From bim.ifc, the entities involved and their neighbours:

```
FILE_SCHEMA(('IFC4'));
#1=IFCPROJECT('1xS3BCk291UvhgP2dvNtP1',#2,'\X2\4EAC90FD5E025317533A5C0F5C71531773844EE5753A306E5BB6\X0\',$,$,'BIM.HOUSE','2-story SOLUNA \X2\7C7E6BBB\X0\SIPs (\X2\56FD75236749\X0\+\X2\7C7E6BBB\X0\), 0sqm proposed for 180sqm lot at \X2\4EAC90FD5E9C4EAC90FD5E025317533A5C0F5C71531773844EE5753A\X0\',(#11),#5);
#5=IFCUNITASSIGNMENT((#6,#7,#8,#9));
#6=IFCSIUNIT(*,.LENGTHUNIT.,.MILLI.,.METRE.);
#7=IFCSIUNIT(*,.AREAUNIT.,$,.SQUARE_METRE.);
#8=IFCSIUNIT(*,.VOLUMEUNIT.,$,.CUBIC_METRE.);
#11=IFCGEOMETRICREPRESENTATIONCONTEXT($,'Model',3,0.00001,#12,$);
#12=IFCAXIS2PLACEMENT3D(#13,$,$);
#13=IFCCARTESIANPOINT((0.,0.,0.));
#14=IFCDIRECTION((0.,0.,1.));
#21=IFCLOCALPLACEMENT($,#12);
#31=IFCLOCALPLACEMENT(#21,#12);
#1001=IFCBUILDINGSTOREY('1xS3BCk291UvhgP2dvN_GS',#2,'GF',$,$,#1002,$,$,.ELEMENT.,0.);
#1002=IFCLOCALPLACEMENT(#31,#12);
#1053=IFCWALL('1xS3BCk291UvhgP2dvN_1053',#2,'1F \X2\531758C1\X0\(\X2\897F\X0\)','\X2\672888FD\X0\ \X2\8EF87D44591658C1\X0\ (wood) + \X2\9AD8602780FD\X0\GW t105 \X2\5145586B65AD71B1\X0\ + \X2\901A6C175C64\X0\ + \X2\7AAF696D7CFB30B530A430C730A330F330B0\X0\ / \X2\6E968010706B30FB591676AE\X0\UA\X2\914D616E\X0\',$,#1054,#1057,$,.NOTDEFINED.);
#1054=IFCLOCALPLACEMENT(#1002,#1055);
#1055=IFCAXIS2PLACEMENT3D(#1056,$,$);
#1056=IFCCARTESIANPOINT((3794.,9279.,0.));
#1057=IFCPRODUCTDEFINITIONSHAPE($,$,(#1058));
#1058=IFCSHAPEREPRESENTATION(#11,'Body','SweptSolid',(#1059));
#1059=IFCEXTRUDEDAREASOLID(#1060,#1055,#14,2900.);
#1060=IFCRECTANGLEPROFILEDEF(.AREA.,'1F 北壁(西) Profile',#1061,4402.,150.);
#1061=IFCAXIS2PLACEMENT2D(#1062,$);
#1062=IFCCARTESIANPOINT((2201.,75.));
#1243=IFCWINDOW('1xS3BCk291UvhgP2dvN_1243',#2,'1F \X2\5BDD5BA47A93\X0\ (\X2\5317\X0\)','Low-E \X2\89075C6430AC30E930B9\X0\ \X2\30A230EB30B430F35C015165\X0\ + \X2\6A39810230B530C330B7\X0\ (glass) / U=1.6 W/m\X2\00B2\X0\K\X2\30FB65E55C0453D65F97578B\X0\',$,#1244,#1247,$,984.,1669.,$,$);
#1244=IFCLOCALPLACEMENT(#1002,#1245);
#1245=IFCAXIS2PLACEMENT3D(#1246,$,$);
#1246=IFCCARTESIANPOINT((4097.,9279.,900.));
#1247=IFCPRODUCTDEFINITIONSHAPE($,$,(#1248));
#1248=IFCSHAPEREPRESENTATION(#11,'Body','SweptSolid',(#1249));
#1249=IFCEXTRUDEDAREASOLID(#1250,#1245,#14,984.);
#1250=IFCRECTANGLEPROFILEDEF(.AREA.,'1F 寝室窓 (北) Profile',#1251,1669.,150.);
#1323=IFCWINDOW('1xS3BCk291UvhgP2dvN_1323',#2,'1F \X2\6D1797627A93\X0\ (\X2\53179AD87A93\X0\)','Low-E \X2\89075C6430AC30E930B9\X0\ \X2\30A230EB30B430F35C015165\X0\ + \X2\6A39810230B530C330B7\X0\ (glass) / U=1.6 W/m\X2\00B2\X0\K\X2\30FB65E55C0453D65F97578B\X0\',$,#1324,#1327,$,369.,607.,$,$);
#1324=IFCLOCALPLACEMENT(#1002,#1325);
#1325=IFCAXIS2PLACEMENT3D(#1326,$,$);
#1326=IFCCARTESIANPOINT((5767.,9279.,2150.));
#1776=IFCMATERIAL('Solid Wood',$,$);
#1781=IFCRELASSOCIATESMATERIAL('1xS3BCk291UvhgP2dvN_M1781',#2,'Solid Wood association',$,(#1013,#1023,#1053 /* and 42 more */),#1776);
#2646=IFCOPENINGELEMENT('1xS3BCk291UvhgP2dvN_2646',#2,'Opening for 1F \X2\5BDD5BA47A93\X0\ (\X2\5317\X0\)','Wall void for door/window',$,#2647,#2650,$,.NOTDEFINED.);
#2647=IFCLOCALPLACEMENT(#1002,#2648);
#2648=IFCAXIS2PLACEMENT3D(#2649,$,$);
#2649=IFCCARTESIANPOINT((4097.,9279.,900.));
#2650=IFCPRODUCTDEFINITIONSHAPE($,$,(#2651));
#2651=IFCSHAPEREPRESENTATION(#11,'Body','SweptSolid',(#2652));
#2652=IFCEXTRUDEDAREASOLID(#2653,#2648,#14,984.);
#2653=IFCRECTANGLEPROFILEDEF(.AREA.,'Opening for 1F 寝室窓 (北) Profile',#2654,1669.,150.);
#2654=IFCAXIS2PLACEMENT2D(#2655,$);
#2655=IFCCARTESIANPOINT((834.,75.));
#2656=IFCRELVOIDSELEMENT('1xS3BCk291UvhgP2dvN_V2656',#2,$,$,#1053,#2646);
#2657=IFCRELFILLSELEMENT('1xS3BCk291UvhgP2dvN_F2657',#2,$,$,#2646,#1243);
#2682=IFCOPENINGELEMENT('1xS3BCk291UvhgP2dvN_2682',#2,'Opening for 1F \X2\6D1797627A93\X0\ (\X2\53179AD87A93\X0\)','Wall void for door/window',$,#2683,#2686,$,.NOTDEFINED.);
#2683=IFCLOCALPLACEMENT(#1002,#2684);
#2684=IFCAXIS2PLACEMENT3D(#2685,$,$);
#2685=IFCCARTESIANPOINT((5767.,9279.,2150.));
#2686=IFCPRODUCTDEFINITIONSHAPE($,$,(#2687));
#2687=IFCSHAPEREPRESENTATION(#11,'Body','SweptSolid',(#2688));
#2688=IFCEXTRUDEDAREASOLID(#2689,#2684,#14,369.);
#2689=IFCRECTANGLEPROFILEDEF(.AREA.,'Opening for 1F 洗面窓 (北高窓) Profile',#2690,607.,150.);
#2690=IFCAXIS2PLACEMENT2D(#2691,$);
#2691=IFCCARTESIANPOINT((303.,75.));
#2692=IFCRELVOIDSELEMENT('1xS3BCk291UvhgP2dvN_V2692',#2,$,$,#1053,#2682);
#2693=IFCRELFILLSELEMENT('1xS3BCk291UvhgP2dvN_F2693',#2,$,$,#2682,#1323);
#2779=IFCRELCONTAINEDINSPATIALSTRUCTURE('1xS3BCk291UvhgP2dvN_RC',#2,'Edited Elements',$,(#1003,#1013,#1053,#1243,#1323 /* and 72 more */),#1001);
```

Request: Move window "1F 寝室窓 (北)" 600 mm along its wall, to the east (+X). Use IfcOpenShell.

```python
import ifcopenshell
import ifcopenshell.api.geometry
import ifcopenshell.util.placement
import ifcopenshell.util.unit

model = ifcopenshell.open("bim.ifc")
unit_scale = ifcopenshell.util.unit.calculate_unit_scale(model)

window = model.by_guid("1xS3BCk291UvhgP2dvN_1243")
opening = window.FillsVoids[0].RelatingOpeningElement
wall = opening.VoidsElements[0].RelatingBuildingElement

wall_matrix = ifcopenshell.util.placement.get_local_placement(wall.ObjectPlacement)
shift = wall_matrix[:3, 0] * 0.6 / unit_scale
before = ifcopenshell.util.placement.get_local_placement(window.ObjectPlacement)[:3, 3].copy()

# The window is not placed relative to its opening, so move both.
for product in (opening, window):
    matrix = ifcopenshell.util.placement.get_local_placement(product.ObjectPlacement)
    matrix[:3, 3] += shift
    ifcopenshell.api.geometry.edit_object_placement(model, product=product, matrix=matrix, is_si=False)

after = ifcopenshell.util.placement.get_local_placement(window.ObjectPlacement)[:3, 3]
print("window moved by", (after - before).round(3) + 0.0)

model.write("bim_rev.ifc")
```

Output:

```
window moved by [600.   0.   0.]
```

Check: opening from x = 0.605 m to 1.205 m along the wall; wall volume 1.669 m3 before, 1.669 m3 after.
